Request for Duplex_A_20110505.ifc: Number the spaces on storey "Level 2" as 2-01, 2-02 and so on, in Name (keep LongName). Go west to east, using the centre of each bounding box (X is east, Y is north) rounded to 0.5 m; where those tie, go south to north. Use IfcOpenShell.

First a look at what the model holds.

```python
import ifcopenshell
import ifcopenshell.util.element
import ifcopenshell.util.placement

model = ifcopenshell.open("Duplex_A_20110505.ifc")
print(model.schema)
storey = next(s for s in model.by_type("IfcBuildingStorey") if s.Name == "Level 2")
spaces = [e for e in ifcopenshell.util.element.get_decomposition(storey) if e.is_a("IfcSpace")]
for e in sorted(spaces, key=lambda e: e.id()):
    origin = ifcopenshell.util.placement.get_local_placement(e.ObjectPlacement)[:3, 3]
    print(e.id(), e.Name, e.LongName, origin.round(2) + 0.0, sep=" | ")
```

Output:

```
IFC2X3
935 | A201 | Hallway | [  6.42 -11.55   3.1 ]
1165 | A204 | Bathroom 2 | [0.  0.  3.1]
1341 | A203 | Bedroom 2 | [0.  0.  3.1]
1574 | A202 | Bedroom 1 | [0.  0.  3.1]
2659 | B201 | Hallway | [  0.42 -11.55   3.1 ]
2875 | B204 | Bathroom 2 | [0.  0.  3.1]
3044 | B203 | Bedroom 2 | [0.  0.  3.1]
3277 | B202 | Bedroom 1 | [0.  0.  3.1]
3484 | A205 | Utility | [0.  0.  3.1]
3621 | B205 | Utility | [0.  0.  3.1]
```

```python
import ifcopenshell
import ifcopenshell.geom
import ifcopenshell.util.element
import ifcopenshell.util.shape

model = ifcopenshell.open("Duplex_A_20110505.ifc")
settings = ifcopenshell.geom.settings()
settings.set("use-world-coords", True)


def centre(element):
    shape = ifcopenshell.geom.create_shape(settings, element)
    return ifcopenshell.util.shape.get_bbox_centroid(shape.geometry)


storey = next(s for s in model.by_type("IfcBuildingStorey") if s.Name == "Level 2")
spaces = [e for e in ifcopenshell.util.element.get_decomposition(storey) if e.is_a("IfcSpace")]

# Insertion points can sit at a corner or the storey origin, so sort by the geometry (in metres).
centres = {e: centre(e) for e in spaces}
spaces.sort(key=lambda e: (round(centres[e][0] / 0.5), centres[e][1]))

for i, e in enumerate(spaces, start=1):
    number = f"2-{i:02d}"
    e.Name = number
    print(e.id(), number)

model.write("Duplex_A_20110505_v2.ifc")
```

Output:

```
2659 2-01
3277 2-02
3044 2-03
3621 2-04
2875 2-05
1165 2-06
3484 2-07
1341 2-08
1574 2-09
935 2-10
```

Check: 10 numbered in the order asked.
